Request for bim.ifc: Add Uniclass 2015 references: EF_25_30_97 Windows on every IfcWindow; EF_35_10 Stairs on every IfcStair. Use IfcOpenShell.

First a look at what the model holds.

```python
import ifcopenshell

model = ifcopenshell.open("bim.ifc")
print(model.schema)
print("classifications:", [c.Name for c in model.by_type("IfcClassification")])
for ifc_class in ("IfcDoor", "IfcRoof", "IfcStair", "IfcWall", "IfcWindow"):
    print(ifc_class, len(model.by_type(ifc_class)))
```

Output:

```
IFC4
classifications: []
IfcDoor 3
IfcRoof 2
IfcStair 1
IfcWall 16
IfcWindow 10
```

```python
import ifcopenshell
import ifcopenshell.api.classification

model = ifcopenshell.open("bim.ifc")

system = ifcopenshell.api.classification.add_classification(model, classification="Uniclass 2015")

codes = {
    "IfcWindow": ("EF_25_30_97", "Windows"),
    "IfcStair": ("EF_35_10", "Stairs"),
}
for ifc_class, (code, name) in codes.items():
    products = model.by_type(ifc_class)
    ifcopenshell.api.classification.add_reference(
        model, products=products, classification=system, identification=code, name=name
    )
    print(code, len(products))

model.write("bim_edited.ifc")
```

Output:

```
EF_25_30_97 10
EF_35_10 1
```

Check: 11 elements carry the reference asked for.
